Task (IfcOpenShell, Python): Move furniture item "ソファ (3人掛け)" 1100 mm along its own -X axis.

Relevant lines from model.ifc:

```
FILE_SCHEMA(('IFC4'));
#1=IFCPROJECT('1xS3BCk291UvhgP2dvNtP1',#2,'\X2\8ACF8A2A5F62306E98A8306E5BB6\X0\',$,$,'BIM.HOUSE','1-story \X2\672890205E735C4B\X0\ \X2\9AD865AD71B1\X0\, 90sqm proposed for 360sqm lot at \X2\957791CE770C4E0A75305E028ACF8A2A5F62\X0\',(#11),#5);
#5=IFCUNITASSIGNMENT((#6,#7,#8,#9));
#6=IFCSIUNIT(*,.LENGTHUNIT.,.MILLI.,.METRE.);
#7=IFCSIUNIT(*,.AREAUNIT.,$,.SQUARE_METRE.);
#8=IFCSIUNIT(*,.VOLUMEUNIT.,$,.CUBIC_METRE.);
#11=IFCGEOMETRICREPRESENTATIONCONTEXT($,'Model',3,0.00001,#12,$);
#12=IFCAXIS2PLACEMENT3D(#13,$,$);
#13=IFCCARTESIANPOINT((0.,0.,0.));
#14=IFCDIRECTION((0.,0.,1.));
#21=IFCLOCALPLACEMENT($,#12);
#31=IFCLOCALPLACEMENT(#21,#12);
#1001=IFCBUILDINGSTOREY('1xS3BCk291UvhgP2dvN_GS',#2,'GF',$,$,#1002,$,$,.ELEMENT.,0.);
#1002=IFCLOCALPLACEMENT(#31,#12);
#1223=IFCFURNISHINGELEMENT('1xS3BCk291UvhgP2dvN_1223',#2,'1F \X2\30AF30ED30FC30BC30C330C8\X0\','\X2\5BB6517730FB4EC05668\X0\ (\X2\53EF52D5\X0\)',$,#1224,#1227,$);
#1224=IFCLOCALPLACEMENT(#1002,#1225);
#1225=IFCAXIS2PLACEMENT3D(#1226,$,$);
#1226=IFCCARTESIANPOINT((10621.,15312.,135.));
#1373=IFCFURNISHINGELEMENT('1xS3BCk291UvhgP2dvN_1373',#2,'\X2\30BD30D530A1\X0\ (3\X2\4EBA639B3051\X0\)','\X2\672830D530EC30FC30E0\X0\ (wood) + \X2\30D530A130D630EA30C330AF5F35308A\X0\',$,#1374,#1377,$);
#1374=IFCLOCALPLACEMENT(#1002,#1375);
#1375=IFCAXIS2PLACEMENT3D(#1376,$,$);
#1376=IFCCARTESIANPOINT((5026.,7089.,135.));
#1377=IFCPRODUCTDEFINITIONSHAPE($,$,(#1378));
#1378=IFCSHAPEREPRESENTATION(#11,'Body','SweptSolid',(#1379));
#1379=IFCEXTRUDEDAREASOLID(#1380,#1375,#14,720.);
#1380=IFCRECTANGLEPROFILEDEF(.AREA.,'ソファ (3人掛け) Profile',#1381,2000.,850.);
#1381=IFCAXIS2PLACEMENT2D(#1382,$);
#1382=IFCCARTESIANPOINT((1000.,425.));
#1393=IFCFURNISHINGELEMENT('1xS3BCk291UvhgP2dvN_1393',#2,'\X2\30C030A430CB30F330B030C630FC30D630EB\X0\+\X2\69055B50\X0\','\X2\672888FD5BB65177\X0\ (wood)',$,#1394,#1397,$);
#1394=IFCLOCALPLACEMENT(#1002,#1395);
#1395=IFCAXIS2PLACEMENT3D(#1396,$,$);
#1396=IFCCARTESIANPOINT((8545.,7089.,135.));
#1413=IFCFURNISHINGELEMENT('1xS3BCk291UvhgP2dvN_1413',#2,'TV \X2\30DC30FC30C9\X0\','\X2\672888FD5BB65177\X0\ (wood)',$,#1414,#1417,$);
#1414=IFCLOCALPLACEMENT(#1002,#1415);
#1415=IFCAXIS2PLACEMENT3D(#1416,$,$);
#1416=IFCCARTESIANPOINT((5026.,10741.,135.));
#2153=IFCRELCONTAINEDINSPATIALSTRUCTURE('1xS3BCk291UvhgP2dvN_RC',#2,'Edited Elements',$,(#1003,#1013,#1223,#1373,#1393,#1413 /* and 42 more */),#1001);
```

```python
import ifcopenshell
import ifcopenshell.api.geometry
import ifcopenshell.util.placement

model = ifcopenshell.open("model.ifc")

item = model.by_id(1373)
matrix = ifcopenshell.util.placement.get_local_placement(item.ObjectPlacement)
matrix[:3, 3] -= matrix[:3, 0] * 1100.0
ifcopenshell.api.geometry.edit_object_placement(model, product=item, matrix=matrix, is_si=False)

print(ifcopenshell.util.placement.get_local_placement(item.ObjectPlacement).round(3) + 0.0)

model.write("model_updated.ifc")
```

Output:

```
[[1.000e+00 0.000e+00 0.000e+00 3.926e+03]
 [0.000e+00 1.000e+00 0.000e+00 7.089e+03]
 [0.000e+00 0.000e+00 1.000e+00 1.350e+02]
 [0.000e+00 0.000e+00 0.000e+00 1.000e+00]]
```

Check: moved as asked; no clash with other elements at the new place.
